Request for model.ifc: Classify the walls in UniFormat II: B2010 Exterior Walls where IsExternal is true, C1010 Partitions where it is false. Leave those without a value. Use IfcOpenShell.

First a look at what the model holds.

```python
import ifcopenshell
import ifcopenshell.util.element

model = ifcopenshell.open("model.ifc")
print(model.schema)
print("classifications:", [c.Name for c in model.by_type("IfcClassification")])
values = [ifcopenshell.util.element.get_pset(e, "Pset_WallCommon", "IsExternal") for e in model.by_type("IfcWall")]
for value in (True, False, None):
    print("IsExternal", value, values.count(value))
```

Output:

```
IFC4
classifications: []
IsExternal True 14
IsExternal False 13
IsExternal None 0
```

```python
import ifcopenshell
import ifcopenshell.api.classification
import ifcopenshell.util.element

model = ifcopenshell.open("model.ifc")

system = ifcopenshell.api.classification.add_classification(model, classification="UniFormat II")

walls = model.by_type("IfcWall")
external = {e: ifcopenshell.util.element.get_pset(e, "Pset_WallCommon", "IsExternal") for e in walls}
for flag, code, name in ((True, "B2010", "Exterior Walls"), (False, "C1010", "Partitions")):
    products = [e for e in walls if external[e] is flag]
    ifcopenshell.api.classification.add_reference(
        model, products=products, classification=system, identification=code, name=name
    )
    print(code, len(products))

model.write("model_v2.ifc")
```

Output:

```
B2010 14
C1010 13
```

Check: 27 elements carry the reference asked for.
